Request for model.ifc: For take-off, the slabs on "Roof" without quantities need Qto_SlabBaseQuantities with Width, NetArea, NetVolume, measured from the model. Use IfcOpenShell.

First a look at what the model holds.

```python
import ifcopenshell
import ifcopenshell.util.element
import ifcopenshell.util.unit

model = ifcopenshell.open("model.ifc")
print(model.schema)
for unit_type in ("LENGTHUNIT", "AREAUNIT", "VOLUMEUNIT"):
    print(unit_type, ifcopenshell.util.unit.calculate_unit_scale(model, unit_type))
storey = next(s for s in model.by_type("IfcBuildingStorey") if s.Name == "Roof")
slabs = [e for e in ifcopenshell.util.element.get_decomposition(storey) if e.is_a("IfcSlab")]
for e in sorted(slabs, key=lambda e: e.id()):
    print(e.id(), e.is_a(), e.Name, list(ifcopenshell.util.element.get_psets(e, qtos_only=True)), sep=" | ")
```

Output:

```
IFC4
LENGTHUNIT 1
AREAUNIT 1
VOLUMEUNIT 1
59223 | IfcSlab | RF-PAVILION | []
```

```python
import ifcopenshell
import ifcopenshell.api.pset
import ifcopenshell.geom
import ifcopenshell.util.element
import ifcopenshell.util.shape
import ifcopenshell.util.unit

model = ifcopenshell.open("model.ifc")
unit_scale = ifcopenshell.util.unit.calculate_unit_scale(model)
area_scale = ifcopenshell.util.unit.calculate_unit_scale(model, "AREAUNIT")
volume_scale = ifcopenshell.util.unit.calculate_unit_scale(model, "VOLUMEUNIT")
settings = ifcopenshell.geom.settings()

storey = next(s for s in model.by_type("IfcBuildingStorey") if s.Name == "Roof")
slabs = [e for e in ifcopenshell.util.element.get_decomposition(storey) if e.is_a("IfcSlab")]

for e in sorted(slabs, key=lambda e: e.id()):
    if ifcopenshell.util.element.get_psets(e, qtos_only=True, should_inherit=False):
        continue
    # Geometry comes back in metres, in the element's own axes.
    shape = ifcopenshell.geom.create_shape(settings, e)
    values = {
        "Width": ifcopenshell.util.shape.get_z(shape.geometry) / unit_scale,
        "NetArea": ifcopenshell.util.shape.get_footprint_area(shape.geometry) / area_scale,
        "NetVolume": ifcopenshell.util.shape.get_volume(shape.geometry) / volume_scale,
    }
    qto = ifcopenshell.api.pset.add_qto(model, product=e, name="Qto_SlabBaseQuantities")
    ifcopenshell.api.pset.edit_qto(model, qto=qto, properties=values)
    print(e.id(), {k: round(v, 3) for k, v in values.items()})

model.write("model-out.ifc")
```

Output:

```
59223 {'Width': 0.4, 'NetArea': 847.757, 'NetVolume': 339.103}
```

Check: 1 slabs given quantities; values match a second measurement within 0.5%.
